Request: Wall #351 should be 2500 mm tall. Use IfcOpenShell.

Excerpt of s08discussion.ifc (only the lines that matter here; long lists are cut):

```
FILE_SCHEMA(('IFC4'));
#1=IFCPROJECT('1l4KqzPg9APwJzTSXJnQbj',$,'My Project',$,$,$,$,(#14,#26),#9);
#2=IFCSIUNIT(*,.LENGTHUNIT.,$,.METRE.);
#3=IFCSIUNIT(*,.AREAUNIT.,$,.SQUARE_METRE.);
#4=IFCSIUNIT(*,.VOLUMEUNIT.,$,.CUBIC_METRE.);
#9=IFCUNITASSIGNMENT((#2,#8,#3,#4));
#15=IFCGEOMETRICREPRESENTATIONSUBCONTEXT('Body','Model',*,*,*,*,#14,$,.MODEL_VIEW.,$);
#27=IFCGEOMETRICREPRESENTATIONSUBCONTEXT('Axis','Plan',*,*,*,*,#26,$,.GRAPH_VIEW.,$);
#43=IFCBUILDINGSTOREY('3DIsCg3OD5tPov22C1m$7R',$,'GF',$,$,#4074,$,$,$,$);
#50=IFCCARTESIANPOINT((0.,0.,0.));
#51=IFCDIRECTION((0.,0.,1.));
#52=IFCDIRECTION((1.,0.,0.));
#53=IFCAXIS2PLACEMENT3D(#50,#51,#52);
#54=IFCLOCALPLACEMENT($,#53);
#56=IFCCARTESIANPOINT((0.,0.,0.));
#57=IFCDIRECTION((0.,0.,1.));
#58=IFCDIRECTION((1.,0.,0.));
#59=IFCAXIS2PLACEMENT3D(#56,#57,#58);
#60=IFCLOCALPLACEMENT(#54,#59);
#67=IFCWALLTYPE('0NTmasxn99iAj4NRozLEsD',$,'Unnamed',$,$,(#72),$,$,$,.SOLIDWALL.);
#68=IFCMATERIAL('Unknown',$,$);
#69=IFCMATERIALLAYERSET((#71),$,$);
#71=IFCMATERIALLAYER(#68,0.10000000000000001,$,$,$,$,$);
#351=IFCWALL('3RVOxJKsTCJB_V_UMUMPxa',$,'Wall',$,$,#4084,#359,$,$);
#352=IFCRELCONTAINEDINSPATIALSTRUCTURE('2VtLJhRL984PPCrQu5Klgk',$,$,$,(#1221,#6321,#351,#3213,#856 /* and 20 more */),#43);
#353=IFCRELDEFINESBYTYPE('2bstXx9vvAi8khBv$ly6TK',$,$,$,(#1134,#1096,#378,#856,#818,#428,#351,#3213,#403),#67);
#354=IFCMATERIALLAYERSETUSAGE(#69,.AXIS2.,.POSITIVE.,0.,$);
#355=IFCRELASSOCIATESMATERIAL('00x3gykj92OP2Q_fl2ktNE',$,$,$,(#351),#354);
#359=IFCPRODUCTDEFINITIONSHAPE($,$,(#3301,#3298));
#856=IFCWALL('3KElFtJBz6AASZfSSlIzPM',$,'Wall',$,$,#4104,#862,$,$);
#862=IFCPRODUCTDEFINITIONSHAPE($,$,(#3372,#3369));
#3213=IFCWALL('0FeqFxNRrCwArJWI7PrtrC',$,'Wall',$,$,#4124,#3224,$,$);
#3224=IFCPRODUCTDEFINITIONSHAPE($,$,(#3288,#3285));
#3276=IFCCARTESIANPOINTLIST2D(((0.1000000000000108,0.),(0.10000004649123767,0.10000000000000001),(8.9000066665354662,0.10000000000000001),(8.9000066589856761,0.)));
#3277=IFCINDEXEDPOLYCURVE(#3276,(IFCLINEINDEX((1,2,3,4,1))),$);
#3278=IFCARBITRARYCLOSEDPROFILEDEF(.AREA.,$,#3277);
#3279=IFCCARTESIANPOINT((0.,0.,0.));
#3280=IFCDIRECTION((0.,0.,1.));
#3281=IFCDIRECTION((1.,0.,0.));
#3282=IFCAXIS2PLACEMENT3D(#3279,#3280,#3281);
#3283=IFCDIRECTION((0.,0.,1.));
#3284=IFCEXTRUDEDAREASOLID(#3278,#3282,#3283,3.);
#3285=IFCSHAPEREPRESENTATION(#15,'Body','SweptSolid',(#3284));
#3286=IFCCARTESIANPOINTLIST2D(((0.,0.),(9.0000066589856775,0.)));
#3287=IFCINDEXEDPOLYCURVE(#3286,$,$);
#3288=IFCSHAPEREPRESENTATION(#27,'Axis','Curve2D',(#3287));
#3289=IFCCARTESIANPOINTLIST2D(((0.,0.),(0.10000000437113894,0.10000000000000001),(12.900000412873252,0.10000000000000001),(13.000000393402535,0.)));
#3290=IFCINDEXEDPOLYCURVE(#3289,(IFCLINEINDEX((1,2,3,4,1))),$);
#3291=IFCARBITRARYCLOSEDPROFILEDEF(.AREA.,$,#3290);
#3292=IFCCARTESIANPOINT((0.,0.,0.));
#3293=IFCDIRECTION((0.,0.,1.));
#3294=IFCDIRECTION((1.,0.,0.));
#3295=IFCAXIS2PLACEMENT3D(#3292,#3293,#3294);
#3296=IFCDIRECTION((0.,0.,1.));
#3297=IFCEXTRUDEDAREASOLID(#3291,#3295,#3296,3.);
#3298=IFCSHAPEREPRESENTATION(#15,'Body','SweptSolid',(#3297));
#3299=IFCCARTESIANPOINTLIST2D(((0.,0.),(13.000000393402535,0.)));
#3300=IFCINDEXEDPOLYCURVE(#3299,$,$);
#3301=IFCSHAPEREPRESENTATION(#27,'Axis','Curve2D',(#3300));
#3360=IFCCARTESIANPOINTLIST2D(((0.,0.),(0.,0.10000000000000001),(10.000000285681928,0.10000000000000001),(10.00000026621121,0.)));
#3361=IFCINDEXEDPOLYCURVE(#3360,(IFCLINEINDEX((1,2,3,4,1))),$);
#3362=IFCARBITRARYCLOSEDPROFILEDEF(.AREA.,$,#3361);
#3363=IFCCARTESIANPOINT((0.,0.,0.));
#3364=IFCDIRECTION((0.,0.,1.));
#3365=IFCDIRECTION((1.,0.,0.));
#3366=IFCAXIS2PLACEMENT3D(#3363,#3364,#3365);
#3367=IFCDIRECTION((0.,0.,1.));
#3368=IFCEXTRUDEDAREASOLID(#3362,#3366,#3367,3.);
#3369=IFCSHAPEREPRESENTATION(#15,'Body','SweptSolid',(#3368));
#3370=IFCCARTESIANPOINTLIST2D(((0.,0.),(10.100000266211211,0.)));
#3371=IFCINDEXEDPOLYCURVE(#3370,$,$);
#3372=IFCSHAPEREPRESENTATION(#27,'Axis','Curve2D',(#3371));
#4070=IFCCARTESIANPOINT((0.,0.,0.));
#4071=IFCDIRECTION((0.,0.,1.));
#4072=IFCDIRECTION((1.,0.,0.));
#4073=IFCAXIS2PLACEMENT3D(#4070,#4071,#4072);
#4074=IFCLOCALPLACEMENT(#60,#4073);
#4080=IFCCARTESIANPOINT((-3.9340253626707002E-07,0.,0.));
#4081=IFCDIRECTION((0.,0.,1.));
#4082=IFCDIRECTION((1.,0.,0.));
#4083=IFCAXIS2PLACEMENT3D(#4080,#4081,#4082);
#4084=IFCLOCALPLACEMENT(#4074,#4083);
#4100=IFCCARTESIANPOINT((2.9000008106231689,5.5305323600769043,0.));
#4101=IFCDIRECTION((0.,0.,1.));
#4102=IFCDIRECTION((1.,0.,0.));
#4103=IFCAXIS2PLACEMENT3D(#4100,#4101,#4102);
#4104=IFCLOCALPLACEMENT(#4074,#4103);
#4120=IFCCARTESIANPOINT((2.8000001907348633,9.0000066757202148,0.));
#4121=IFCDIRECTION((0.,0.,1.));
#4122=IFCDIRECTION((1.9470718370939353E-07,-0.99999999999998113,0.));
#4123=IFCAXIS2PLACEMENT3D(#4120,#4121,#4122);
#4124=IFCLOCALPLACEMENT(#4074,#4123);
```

```python
import ifcopenshell
import ifcopenshell.geom
import ifcopenshell.util.representation
import ifcopenshell.util.shape
import ifcopenshell.util.unit

model = ifcopenshell.open("s08discussion.ifc")
unit_scale = ifcopenshell.util.unit.calculate_unit_scale(model)
settings = ifcopenshell.geom.settings()


def volume(element):
    """Net volume in cubic metres, openings subtracted."""
    shape = ifcopenshell.geom.create_shape(settings, element)
    return ifcopenshell.util.shape.get_volume(shape.geometry)


wall = model.by_guid("3RVOxJKsTCJB_V_UMUMPxa")
before = volume(wall)

body = ifcopenshell.util.representation.get_representation(wall, "Model", "Body")
solid = body.Items[0]
old_height = solid.Depth
solid.Depth = 2.5 / unit_scale
after = volume(wall)

print(f"height {old_height:g} -> {solid.Depth:g}, volume {before:.3f} -> {after:.3f} m3")

model.write("s08discussion_updated.ifc")
```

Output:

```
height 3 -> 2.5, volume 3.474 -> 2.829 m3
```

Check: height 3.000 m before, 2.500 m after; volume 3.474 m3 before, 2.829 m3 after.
